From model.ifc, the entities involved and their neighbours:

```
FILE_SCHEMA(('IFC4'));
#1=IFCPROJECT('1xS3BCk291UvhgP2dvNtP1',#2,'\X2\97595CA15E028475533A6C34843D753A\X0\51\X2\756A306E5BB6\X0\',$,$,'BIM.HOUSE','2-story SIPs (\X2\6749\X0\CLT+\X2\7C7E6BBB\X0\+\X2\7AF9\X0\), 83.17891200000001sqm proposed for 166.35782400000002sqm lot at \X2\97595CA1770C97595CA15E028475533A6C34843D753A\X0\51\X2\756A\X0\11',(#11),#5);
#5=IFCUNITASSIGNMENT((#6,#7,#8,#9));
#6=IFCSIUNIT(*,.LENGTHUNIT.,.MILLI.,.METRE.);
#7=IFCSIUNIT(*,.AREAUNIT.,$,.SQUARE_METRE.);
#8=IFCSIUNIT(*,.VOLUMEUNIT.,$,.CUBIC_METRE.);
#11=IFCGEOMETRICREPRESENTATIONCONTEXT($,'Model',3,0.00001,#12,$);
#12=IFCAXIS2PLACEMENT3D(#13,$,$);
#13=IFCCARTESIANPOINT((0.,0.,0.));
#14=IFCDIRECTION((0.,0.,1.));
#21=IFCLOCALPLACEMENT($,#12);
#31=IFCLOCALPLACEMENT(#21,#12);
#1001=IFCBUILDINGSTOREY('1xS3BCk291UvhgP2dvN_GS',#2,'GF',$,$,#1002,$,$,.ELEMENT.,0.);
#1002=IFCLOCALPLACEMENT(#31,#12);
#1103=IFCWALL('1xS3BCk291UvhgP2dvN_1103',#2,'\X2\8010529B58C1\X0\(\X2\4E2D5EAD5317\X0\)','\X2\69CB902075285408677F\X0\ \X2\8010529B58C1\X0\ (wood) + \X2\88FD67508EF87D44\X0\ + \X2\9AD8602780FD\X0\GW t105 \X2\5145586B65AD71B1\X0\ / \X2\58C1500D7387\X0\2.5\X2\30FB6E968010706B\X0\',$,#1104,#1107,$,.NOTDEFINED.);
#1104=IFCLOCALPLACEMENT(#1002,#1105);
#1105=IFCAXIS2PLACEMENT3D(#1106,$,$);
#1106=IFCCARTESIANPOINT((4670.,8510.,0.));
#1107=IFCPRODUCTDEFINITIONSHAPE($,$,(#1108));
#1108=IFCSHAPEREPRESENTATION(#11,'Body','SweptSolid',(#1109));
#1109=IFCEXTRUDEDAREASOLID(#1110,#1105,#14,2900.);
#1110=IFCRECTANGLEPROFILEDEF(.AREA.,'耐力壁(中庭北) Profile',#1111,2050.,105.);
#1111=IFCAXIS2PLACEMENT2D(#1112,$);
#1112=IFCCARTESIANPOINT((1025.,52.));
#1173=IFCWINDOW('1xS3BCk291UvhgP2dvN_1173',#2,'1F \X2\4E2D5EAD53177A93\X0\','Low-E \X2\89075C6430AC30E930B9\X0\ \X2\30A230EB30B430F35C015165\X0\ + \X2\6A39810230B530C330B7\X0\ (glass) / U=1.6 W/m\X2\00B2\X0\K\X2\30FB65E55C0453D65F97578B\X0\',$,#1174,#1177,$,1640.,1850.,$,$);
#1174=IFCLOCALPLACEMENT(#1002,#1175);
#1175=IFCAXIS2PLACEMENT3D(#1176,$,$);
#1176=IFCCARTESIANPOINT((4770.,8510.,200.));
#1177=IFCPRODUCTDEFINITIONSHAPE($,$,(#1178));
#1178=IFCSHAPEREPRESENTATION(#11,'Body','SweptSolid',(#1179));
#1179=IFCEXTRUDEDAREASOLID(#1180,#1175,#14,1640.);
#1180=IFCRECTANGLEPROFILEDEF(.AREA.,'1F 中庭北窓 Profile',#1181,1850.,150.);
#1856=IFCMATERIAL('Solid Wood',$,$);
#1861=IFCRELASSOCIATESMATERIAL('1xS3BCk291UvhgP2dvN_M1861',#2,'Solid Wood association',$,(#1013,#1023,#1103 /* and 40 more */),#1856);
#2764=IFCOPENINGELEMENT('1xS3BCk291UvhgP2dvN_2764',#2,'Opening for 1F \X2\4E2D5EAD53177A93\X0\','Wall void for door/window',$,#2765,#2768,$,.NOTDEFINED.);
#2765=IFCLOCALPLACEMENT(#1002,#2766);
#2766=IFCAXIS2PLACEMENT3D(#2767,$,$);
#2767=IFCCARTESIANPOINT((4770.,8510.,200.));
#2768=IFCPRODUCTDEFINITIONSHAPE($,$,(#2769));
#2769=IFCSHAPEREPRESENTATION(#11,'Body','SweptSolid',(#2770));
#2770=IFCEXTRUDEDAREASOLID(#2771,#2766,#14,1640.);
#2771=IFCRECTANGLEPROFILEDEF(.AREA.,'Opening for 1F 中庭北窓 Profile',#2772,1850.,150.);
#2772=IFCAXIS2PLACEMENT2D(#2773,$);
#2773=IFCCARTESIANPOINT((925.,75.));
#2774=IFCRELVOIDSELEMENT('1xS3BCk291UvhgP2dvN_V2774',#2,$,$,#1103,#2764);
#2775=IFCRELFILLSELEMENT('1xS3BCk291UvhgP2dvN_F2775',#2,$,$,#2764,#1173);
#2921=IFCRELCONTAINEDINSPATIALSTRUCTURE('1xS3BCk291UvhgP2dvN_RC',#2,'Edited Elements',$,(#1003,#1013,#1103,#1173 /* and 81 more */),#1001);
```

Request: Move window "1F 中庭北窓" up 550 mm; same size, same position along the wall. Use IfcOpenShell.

```python
import numpy as np
import ifcopenshell
import ifcopenshell.api.geometry
import ifcopenshell.util.placement
import ifcopenshell.util.unit

model = ifcopenshell.open("model.ifc")
unit_scale = ifcopenshell.util.unit.calculate_unit_scale(model)

window = model.by_guid("1xS3BCk291UvhgP2dvN_1173")
opening = window.FillsVoids[0].RelatingOpeningElement
dz = 550.0

shift = np.array([0.0, 0.0, dz])
# The window is not placed relative to its opening, so move both.
for product in (opening, window):
    matrix = ifcopenshell.util.placement.get_local_placement(product.ObjectPlacement)
    matrix[:3, 3] += shift
    ifcopenshell.api.geometry.edit_object_placement(model, product=product, matrix=matrix, is_si=False)

print(f"moved by {dz * unit_scale:+.3f} m")

model.write("model_updated.ifc")
```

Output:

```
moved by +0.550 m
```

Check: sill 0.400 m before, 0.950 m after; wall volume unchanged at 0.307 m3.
